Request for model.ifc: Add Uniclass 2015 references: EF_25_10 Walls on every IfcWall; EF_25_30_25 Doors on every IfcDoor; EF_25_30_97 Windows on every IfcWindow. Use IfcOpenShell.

First a look at what the model holds.

```python
import ifcopenshell

model = ifcopenshell.open("model.ifc")
print(model.schema)
print("classifications:", [c.Name for c in model.by_type("IfcClassification")])
for ifc_class in ("IfcDoor", "IfcRoof", "IfcStair", "IfcWall", "IfcWindow"):
    print(ifc_class, len(model.by_type(ifc_class)))
```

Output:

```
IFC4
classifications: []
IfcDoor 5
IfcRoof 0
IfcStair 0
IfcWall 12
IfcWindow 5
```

```python
import ifcopenshell
import ifcopenshell.api.classification

model = ifcopenshell.open("model.ifc")

system = ifcopenshell.api.classification.add_classification(model, classification="Uniclass 2015")

codes = {
    "IfcWall": ("EF_25_10", "Walls"),
    "IfcDoor": ("EF_25_30_25", "Doors"),
    "IfcWindow": ("EF_25_30_97", "Windows"),
}
for ifc_class, (code, name) in codes.items():
    products = model.by_type(ifc_class)
    ifcopenshell.api.classification.add_reference(
        model, products=products, classification=system, identification=code, name=name
    )
    print(code, len(products))

model.write("model_rev.ifc")
```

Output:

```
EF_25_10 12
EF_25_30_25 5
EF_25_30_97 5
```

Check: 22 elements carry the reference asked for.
